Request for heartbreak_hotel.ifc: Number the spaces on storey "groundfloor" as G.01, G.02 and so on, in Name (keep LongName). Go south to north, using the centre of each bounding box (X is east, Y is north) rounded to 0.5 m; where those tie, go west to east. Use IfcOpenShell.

First a look at what the model holds.

```python
import ifcopenshell
import ifcopenshell.util.element
import ifcopenshell.util.placement

model = ifcopenshell.open("heartbreak_hotel.ifc")
print(model.schema)
storey = next(s for s in model.by_type("IfcBuildingStorey") if s.Name == "groundfloor")
spaces = [e for e in ifcopenshell.util.element.get_decomposition(storey) if e.is_a("IfcSpace")]
for e in sorted(spaces, key=lambda e: e.id()):
    origin = ifcopenshell.util.placement.get_local_placement(e.ObjectPlacement)[:3, 3]
    print(e.id(), e.Name, e.LongName, origin.round(2) + 0.0, sep=" | ")
```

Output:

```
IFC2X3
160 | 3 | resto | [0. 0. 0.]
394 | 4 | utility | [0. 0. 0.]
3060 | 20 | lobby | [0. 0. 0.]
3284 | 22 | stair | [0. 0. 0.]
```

```python
import ifcopenshell
import ifcopenshell.geom
import ifcopenshell.util.element
import ifcopenshell.util.shape

model = ifcopenshell.open("heartbreak_hotel.ifc")
settings = ifcopenshell.geom.settings()
settings.set("use-world-coords", True)


def centre(element):
    shape = ifcopenshell.geom.create_shape(settings, element)
    return ifcopenshell.util.shape.get_bbox_centroid(shape.geometry)


storey = next(s for s in model.by_type("IfcBuildingStorey") if s.Name == "groundfloor")
spaces = [e for e in ifcopenshell.util.element.get_decomposition(storey) if e.is_a("IfcSpace")]

# Insertion points can sit at a corner or the storey origin, so sort by the geometry (in metres).
centres = {e: centre(e) for e in spaces}
spaces.sort(key=lambda e: (round(centres[e][1] / 0.5), centres[e][0]))

for i, e in enumerate(spaces, start=1):
    number = f"G.{i:02d}"
    e.Name = number
    print(e.id(), number)

model.write("heartbreak_hotel-out.ifc")
```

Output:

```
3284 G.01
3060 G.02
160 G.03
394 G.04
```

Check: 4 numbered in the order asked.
